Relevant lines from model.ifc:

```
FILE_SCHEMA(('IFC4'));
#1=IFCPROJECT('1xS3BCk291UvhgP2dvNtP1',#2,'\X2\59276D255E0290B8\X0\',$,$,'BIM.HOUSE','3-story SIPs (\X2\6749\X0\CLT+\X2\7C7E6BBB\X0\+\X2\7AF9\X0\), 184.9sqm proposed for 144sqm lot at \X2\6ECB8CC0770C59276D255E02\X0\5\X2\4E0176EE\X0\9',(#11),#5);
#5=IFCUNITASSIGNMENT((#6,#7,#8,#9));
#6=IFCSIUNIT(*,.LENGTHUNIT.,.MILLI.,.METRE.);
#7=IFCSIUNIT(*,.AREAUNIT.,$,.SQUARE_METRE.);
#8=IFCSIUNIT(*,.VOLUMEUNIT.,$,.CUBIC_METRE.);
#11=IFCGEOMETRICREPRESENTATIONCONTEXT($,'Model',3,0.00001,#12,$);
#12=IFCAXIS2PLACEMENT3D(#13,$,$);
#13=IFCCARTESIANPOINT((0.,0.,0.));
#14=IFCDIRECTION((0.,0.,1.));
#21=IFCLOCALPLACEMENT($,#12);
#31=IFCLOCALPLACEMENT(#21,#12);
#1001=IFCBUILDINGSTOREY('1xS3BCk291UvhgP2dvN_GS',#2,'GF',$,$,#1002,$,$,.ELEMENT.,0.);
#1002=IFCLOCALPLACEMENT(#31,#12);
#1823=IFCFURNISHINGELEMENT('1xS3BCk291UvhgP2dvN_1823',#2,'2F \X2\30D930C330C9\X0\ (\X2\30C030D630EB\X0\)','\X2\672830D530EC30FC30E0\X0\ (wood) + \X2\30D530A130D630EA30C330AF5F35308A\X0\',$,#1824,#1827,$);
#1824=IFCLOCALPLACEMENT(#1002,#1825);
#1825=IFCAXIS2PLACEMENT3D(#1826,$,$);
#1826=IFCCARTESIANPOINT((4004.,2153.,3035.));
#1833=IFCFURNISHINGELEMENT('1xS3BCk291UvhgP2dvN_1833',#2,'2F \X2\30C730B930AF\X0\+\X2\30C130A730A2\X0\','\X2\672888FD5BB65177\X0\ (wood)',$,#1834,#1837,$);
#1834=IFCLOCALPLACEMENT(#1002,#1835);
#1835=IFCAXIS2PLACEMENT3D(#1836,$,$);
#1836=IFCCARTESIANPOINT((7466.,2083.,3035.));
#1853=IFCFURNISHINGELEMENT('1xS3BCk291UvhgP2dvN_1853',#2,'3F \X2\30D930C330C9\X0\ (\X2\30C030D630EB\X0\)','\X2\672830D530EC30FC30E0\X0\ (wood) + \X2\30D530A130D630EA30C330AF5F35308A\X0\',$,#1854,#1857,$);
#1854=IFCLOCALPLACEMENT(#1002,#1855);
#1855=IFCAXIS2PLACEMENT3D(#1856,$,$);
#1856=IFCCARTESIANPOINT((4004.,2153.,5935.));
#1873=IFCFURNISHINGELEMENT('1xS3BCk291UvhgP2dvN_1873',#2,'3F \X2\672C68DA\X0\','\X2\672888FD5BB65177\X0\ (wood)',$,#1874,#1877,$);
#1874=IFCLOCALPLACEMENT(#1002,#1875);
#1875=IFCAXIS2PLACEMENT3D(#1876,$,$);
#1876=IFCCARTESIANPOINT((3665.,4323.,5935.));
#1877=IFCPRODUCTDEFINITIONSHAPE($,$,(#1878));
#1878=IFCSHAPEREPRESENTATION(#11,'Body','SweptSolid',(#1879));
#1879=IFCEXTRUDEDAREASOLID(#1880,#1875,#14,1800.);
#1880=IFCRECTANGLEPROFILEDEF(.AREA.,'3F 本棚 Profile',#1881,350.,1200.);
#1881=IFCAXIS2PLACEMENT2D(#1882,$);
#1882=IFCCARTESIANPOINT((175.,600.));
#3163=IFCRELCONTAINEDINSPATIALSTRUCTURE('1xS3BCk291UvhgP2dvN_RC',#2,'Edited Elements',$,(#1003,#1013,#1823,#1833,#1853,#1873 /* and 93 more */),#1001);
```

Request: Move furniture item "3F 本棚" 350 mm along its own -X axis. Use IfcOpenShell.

```python
import ifcopenshell
import ifcopenshell.api.geometry
import ifcopenshell.util.placement
import ifcopenshell.util.unit

model = ifcopenshell.open("model.ifc")
unit_scale = ifcopenshell.util.unit.calculate_unit_scale(model)

item = model.by_guid("1xS3BCk291UvhgP2dvN_1873")
matrix = ifcopenshell.util.placement.get_local_placement(item.ObjectPlacement)
matrix[:3, 3] -= matrix[:3, 0] * 0.35 / unit_scale
ifcopenshell.api.geometry.edit_object_placement(model, product=item, matrix=matrix, is_si=False)

print(ifcopenshell.util.placement.get_local_placement(item.ObjectPlacement).round(3) + 0.0)

model.write("model_edited.ifc")
```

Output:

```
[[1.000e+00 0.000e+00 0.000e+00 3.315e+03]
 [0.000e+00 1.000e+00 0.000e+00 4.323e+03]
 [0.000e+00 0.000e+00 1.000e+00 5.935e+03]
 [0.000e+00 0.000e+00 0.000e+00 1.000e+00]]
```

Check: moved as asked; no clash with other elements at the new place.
